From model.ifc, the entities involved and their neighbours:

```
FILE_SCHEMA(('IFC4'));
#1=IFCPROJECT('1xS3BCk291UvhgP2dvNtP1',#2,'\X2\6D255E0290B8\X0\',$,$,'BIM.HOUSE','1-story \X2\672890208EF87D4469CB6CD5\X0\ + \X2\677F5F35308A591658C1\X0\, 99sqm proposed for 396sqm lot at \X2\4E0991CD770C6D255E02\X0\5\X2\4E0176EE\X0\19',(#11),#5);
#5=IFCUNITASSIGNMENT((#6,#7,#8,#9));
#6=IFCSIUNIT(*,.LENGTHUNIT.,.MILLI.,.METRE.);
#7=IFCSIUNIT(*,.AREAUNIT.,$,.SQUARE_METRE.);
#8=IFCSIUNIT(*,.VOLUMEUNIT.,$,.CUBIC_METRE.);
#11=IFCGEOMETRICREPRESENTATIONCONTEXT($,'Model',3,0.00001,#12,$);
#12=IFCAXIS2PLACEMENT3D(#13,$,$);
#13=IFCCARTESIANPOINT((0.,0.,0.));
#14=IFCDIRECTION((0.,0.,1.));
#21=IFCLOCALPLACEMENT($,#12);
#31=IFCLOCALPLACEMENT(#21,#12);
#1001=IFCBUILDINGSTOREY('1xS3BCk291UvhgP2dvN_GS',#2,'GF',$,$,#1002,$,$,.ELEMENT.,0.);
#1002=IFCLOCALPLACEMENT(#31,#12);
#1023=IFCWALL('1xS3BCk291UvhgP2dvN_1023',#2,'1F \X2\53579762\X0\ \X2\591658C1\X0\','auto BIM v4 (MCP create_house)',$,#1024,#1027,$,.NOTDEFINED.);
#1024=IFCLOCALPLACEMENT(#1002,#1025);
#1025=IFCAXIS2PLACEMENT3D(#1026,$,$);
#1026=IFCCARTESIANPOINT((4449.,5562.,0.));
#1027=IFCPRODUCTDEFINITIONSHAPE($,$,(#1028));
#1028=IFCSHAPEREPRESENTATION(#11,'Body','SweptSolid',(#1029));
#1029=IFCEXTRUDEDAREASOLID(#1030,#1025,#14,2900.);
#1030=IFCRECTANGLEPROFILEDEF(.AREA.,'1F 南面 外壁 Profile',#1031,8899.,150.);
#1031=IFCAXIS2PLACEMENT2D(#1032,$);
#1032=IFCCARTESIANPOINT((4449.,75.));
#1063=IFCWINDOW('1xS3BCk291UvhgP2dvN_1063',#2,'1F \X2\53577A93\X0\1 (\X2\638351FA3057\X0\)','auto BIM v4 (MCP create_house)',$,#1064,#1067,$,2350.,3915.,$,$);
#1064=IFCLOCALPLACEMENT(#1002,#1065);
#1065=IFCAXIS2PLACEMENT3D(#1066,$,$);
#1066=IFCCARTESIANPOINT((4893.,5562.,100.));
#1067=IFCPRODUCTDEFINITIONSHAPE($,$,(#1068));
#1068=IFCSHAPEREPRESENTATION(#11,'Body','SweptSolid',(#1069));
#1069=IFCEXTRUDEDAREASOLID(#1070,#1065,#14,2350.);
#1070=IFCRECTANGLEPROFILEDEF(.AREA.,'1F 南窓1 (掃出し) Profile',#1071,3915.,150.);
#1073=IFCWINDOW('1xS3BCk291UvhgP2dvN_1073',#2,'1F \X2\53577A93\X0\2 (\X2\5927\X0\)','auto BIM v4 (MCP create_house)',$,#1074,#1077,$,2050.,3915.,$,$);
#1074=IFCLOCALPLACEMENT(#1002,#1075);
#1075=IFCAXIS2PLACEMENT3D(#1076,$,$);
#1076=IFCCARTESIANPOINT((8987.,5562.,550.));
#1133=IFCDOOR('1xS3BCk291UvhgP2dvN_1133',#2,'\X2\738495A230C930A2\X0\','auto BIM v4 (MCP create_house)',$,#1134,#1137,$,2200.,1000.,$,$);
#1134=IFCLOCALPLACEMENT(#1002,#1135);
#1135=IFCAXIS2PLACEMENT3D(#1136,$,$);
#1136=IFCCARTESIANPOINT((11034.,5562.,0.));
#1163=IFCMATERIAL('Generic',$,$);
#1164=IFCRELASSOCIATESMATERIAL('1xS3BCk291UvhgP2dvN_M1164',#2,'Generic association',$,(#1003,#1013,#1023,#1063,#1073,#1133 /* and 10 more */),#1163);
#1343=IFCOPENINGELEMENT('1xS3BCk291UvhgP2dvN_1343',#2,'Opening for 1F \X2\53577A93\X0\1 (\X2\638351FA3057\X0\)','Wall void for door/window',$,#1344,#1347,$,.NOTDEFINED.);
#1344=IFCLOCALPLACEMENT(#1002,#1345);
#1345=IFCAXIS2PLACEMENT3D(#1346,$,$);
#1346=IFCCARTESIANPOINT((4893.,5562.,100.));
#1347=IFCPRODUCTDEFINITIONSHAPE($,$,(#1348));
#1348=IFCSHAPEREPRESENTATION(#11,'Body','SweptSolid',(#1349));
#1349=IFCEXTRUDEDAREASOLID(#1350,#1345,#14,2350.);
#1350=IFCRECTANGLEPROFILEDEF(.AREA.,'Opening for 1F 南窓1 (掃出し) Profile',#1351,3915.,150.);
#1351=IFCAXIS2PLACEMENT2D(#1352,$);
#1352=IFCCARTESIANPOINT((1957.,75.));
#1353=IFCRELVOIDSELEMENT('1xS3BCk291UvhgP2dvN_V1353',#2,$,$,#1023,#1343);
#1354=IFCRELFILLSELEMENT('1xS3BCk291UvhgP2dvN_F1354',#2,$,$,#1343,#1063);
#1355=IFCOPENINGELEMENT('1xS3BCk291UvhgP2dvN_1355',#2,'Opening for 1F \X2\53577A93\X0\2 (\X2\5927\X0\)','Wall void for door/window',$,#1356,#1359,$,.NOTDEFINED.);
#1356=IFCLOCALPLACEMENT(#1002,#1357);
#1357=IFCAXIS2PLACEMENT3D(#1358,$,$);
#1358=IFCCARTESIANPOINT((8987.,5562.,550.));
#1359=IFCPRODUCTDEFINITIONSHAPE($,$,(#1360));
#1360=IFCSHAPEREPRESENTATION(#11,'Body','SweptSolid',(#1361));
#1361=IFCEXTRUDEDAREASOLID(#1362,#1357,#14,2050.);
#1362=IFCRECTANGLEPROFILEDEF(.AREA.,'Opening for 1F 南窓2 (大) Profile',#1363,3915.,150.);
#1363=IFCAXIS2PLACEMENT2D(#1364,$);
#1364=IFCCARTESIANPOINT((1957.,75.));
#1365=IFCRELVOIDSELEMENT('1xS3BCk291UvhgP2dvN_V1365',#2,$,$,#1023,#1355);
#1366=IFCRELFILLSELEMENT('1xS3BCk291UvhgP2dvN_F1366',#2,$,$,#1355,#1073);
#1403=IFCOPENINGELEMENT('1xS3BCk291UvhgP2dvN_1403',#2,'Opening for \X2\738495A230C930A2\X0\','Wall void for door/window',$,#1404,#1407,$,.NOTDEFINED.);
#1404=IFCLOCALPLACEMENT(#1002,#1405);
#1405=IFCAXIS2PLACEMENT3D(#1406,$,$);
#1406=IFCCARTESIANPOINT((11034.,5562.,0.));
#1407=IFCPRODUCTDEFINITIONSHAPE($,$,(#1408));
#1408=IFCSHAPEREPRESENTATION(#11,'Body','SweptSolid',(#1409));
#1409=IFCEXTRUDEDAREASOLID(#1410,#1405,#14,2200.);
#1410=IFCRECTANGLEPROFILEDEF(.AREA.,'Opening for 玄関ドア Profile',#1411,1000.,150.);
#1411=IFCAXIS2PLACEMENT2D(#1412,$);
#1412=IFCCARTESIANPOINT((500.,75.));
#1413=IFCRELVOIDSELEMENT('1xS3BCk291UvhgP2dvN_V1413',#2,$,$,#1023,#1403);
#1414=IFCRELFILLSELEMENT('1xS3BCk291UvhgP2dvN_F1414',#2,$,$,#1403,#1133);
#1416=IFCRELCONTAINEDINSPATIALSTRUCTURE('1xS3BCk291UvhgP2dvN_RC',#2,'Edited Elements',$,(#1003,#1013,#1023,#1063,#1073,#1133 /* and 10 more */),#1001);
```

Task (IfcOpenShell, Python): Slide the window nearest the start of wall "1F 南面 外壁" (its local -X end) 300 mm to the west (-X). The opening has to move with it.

```python
import ifcopenshell
import ifcopenshell.api.geometry
import ifcopenshell.util.placement
import ifcopenshell.util.unit

model = ifcopenshell.open("model.ifc")
unit_scale = ifcopenshell.util.unit.calculate_unit_scale(model)

window = model.by_guid("1xS3BCk291UvhgP2dvN_1063")
opening = window.FillsVoids[0].RelatingOpeningElement
wall = opening.VoidsElements[0].RelatingBuildingElement

wall_matrix = ifcopenshell.util.placement.get_local_placement(wall.ObjectPlacement)
shift = wall_matrix[:3, 0] * -0.3 / unit_scale
before = ifcopenshell.util.placement.get_local_placement(window.ObjectPlacement)[:3, 3].copy()

# The window is not placed relative to its opening, so move both.
for product in (opening, window):
    matrix = ifcopenshell.util.placement.get_local_placement(product.ObjectPlacement)
    matrix[:3, 3] += shift
    ifcopenshell.api.geometry.edit_object_placement(model, product=product, matrix=matrix, is_si=False)

after = ifcopenshell.util.placement.get_local_placement(window.ObjectPlacement)[:3, 3]
print("window moved by", (after - before).round(3) + 0.0)

model.write("model-out.ifc")
```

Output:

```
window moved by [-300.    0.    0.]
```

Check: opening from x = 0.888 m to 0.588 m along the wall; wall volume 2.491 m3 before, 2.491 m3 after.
